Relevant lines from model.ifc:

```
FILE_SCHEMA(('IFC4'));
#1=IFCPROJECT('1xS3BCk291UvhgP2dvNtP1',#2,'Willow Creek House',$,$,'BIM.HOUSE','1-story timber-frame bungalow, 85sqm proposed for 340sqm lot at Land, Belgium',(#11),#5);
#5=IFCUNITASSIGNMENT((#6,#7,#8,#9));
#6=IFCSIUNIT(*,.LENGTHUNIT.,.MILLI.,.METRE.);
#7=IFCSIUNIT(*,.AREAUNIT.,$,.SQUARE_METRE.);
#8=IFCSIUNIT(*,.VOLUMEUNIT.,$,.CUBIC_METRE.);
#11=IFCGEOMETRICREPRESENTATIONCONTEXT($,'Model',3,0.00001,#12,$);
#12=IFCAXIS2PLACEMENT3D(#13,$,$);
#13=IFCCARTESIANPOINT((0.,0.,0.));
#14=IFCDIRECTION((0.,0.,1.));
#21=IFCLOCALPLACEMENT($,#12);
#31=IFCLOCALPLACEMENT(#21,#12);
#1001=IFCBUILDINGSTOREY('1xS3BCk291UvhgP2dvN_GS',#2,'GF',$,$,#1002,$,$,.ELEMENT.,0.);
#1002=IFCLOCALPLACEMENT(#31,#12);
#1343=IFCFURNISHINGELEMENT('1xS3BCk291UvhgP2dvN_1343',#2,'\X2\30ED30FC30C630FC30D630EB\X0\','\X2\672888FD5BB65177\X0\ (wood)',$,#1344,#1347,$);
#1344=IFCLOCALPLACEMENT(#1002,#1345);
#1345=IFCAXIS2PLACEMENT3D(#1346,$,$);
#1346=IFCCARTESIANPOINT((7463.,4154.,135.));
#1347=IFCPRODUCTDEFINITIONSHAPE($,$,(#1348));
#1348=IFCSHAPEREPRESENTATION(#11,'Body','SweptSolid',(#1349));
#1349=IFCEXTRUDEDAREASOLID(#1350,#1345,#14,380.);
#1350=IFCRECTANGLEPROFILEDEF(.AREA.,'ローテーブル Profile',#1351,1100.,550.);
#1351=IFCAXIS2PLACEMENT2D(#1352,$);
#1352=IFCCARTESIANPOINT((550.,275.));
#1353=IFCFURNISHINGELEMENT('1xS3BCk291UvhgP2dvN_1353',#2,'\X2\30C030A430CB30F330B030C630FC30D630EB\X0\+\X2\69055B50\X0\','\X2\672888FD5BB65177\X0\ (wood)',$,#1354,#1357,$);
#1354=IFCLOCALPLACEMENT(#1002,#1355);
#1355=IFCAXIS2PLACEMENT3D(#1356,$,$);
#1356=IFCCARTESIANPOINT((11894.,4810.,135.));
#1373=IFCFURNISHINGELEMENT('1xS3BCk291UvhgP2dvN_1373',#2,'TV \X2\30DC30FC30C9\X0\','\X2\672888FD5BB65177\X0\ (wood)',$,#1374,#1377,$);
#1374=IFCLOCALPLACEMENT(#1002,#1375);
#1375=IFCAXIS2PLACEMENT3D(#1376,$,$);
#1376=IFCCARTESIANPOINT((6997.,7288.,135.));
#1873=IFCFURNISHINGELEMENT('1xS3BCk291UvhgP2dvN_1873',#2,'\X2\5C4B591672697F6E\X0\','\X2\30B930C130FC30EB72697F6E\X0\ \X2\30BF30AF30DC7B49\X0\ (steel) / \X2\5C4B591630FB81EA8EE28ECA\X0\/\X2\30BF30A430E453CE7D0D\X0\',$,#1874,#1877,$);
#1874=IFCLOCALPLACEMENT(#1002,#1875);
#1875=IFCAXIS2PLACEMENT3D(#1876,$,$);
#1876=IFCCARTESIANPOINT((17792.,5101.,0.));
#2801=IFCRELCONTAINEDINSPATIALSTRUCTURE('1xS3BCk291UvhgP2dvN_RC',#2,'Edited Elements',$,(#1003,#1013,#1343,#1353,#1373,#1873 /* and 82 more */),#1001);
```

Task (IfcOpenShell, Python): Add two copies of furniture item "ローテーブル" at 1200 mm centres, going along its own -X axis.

```python
import ifcopenshell
import ifcopenshell.api.geometry
import ifcopenshell.api.root
import ifcopenshell.util.element
import ifcopenshell.util.placement
import ifcopenshell.util.unit

model = ifcopenshell.open("model.ifc")
unit_scale = ifcopenshell.util.unit.calculate_unit_scale(model)


def reuse_history(source, copy):
    """copy_class also copies each property set's owner history, people and application; keep the originals."""
    for rel in copy.IsDefinedBy:
        if rel.is_a("IfcRelDefinesByProperties") and (history := rel.RelatingPropertyDefinition.OwnerHistory):
            rel.RelatingPropertyDefinition.OwnerHistory = source.OwnerHistory
            ifcopenshell.util.element.remove_deep2(model, history)


source = model.by_id(1343)
base = ifcopenshell.util.placement.get_local_placement(source.ObjectPlacement)
step = -base[:3, 0] * 1.2 / unit_scale

for i in range(1, 3):
    copy = ifcopenshell.api.root.copy_class(model, product=source)
    copy.Representation = ifcopenshell.util.element.copy_deep(
        model, source.Representation, exclude=["IfcGeometricRepresentationContext", "IfcRepresentationMap"]
    )
    reuse_history(source, copy)
    matrix = base.copy()
    matrix[:3, 3] += i * step
    print("added at", matrix[:3, 3].round(3) + 0.0)
    ifcopenshell.api.geometry.edit_object_placement(model, product=copy, matrix=matrix, is_si=False)

model.write("model_updated.ifc")
```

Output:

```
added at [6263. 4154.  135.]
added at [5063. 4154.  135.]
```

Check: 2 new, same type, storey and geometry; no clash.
